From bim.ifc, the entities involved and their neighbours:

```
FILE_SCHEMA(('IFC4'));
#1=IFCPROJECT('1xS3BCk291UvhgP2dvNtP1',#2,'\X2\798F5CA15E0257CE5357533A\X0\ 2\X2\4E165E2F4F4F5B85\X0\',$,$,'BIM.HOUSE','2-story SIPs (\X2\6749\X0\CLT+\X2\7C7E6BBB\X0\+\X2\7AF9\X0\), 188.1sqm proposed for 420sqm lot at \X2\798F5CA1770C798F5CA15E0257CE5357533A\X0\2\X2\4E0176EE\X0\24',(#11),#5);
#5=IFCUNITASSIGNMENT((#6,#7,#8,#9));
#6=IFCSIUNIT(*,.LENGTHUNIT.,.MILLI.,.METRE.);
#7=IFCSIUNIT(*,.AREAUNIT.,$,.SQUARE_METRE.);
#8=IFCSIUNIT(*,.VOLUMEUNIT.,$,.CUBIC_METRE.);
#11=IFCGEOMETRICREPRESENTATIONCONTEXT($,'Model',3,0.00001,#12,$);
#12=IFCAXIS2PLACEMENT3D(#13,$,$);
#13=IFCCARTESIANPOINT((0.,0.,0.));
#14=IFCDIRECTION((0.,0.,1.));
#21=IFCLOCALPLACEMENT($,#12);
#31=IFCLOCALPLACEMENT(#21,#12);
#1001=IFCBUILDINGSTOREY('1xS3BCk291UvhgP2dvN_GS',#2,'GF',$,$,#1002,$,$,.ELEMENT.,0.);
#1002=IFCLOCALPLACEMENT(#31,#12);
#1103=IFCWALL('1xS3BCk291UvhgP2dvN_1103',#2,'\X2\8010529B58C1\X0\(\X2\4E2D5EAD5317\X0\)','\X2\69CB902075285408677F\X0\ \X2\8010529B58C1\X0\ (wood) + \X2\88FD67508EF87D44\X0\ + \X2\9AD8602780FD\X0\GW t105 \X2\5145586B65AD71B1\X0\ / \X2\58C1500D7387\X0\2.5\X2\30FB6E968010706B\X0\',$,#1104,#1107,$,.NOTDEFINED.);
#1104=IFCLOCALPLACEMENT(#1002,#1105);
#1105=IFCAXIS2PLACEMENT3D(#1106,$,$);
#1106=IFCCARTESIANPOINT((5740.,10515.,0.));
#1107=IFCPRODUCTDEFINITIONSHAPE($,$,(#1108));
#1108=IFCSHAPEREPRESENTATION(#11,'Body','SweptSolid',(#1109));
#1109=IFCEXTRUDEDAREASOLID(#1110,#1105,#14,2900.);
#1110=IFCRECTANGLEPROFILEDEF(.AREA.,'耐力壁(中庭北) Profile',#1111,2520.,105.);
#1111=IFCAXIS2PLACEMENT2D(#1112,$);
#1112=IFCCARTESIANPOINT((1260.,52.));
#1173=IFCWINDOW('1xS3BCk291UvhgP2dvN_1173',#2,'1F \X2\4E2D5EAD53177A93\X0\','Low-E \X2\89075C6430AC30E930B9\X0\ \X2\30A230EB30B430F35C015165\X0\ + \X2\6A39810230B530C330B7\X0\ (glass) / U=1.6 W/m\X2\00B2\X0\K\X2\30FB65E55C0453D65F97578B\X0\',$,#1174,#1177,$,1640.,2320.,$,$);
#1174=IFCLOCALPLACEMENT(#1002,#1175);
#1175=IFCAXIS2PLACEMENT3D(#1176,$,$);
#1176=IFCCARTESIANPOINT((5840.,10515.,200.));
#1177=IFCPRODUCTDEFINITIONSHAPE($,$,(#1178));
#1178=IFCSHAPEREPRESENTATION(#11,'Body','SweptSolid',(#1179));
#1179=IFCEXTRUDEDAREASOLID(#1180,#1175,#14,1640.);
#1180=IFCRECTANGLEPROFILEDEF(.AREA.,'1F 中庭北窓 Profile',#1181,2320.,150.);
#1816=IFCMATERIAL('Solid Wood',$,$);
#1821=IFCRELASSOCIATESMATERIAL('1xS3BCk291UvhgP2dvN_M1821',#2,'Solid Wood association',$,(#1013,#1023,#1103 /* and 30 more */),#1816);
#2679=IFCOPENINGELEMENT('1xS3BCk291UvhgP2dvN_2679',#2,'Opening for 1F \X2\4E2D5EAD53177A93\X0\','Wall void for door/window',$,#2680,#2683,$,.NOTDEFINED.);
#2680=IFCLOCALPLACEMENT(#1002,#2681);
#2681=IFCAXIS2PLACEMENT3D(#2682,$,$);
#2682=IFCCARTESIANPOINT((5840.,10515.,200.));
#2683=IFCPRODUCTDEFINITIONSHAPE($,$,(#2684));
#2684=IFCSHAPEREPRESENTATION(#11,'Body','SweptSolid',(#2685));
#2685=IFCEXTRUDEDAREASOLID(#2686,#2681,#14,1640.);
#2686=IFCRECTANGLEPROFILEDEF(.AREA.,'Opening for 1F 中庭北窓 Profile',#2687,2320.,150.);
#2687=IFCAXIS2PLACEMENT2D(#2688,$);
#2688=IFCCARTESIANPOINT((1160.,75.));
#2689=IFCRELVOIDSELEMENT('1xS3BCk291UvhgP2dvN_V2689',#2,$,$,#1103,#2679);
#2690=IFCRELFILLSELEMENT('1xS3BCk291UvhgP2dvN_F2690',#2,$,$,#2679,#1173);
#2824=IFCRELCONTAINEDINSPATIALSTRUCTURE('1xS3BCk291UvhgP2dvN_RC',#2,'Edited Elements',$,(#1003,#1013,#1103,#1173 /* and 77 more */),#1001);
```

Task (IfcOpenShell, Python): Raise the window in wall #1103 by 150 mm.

```python
import numpy as np
import ifcopenshell
import ifcopenshell.api.geometry
import ifcopenshell.util.placement
import ifcopenshell.util.unit

model = ifcopenshell.open("bim.ifc")
unit_scale = ifcopenshell.util.unit.calculate_unit_scale(model)

window = model.by_guid("1xS3BCk291UvhgP2dvN_1173")
opening = window.FillsVoids[0].RelatingOpeningElement
dz = 150.0

shift = np.array([0.0, 0.0, dz])
# The window is not placed relative to its opening, so move both.
for product in (opening, window):
    matrix = ifcopenshell.util.placement.get_local_placement(product.ObjectPlacement)
    matrix[:3, 3] += shift
    ifcopenshell.api.geometry.edit_object_placement(model, product=product, matrix=matrix, is_si=False)

print(f"moved by {dz * unit_scale:+.3f} m")

model.write("bim-out.ifc")
```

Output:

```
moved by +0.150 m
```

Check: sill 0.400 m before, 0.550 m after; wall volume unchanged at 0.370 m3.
